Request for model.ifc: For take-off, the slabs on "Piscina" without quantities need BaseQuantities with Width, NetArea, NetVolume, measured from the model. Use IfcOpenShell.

First a look at what the model holds.

```python
import ifcopenshell
import ifcopenshell.util.element
import ifcopenshell.util.unit

model = ifcopenshell.open("model.ifc")
print(model.schema)
for unit_type in ("LENGTHUNIT", "AREAUNIT", "VOLUMEUNIT"):
    print(unit_type, ifcopenshell.util.unit.calculate_unit_scale(model, unit_type))
storey = next(s for s in model.by_type("IfcBuildingStorey") if s.Name == "Piscina")
slabs = [e for e in ifcopenshell.util.element.get_decomposition(storey) if e.is_a("IfcSlab")]
for e in sorted(slabs, key=lambda e: e.id()):
    print(e.id(), e.is_a(), e.Name, list(ifcopenshell.util.element.get_psets(e, qtos_only=True)), sep=" | ")
```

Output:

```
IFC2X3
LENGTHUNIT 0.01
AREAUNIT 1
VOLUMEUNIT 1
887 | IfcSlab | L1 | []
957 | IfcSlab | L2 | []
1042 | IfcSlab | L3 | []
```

```python
import ifcopenshell
import ifcopenshell.api.pset
import ifcopenshell.geom
import ifcopenshell.util.element
import ifcopenshell.util.shape
import ifcopenshell.util.unit

model = ifcopenshell.open("model.ifc")
unit_scale = ifcopenshell.util.unit.calculate_unit_scale(model)
area_scale = ifcopenshell.util.unit.calculate_unit_scale(model, "AREAUNIT")
volume_scale = ifcopenshell.util.unit.calculate_unit_scale(model, "VOLUMEUNIT")
settings = ifcopenshell.geom.settings()

storey = next(s for s in model.by_type("IfcBuildingStorey") if s.Name == "Piscina")
slabs = [e for e in ifcopenshell.util.element.get_decomposition(storey) if e.is_a("IfcSlab")]

for e in sorted(slabs, key=lambda e: e.id()):
    if ifcopenshell.util.element.get_psets(e, qtos_only=True, should_inherit=False):
        continue
    # Geometry comes back in metres, in the element's own axes.
    shape = ifcopenshell.geom.create_shape(settings, e)
    values = {
        "Width": ifcopenshell.util.shape.get_z(shape.geometry) / unit_scale,
        "NetArea": ifcopenshell.util.shape.get_footprint_area(shape.geometry) / area_scale,
        "NetVolume": ifcopenshell.util.shape.get_volume(shape.geometry) / volume_scale,
    }
    qto = ifcopenshell.api.pset.add_qto(model, product=e, name="BaseQuantities")
    ifcopenshell.api.pset.edit_qto(model, qto=qto, properties=values)
    print(e.id(), {k: round(v, 3) for k, v in values.items()})

model.write("model_updated.ifc")
```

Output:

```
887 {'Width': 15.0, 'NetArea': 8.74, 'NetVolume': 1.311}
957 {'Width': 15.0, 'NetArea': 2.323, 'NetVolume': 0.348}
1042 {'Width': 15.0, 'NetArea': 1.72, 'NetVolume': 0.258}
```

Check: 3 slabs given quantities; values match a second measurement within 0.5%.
